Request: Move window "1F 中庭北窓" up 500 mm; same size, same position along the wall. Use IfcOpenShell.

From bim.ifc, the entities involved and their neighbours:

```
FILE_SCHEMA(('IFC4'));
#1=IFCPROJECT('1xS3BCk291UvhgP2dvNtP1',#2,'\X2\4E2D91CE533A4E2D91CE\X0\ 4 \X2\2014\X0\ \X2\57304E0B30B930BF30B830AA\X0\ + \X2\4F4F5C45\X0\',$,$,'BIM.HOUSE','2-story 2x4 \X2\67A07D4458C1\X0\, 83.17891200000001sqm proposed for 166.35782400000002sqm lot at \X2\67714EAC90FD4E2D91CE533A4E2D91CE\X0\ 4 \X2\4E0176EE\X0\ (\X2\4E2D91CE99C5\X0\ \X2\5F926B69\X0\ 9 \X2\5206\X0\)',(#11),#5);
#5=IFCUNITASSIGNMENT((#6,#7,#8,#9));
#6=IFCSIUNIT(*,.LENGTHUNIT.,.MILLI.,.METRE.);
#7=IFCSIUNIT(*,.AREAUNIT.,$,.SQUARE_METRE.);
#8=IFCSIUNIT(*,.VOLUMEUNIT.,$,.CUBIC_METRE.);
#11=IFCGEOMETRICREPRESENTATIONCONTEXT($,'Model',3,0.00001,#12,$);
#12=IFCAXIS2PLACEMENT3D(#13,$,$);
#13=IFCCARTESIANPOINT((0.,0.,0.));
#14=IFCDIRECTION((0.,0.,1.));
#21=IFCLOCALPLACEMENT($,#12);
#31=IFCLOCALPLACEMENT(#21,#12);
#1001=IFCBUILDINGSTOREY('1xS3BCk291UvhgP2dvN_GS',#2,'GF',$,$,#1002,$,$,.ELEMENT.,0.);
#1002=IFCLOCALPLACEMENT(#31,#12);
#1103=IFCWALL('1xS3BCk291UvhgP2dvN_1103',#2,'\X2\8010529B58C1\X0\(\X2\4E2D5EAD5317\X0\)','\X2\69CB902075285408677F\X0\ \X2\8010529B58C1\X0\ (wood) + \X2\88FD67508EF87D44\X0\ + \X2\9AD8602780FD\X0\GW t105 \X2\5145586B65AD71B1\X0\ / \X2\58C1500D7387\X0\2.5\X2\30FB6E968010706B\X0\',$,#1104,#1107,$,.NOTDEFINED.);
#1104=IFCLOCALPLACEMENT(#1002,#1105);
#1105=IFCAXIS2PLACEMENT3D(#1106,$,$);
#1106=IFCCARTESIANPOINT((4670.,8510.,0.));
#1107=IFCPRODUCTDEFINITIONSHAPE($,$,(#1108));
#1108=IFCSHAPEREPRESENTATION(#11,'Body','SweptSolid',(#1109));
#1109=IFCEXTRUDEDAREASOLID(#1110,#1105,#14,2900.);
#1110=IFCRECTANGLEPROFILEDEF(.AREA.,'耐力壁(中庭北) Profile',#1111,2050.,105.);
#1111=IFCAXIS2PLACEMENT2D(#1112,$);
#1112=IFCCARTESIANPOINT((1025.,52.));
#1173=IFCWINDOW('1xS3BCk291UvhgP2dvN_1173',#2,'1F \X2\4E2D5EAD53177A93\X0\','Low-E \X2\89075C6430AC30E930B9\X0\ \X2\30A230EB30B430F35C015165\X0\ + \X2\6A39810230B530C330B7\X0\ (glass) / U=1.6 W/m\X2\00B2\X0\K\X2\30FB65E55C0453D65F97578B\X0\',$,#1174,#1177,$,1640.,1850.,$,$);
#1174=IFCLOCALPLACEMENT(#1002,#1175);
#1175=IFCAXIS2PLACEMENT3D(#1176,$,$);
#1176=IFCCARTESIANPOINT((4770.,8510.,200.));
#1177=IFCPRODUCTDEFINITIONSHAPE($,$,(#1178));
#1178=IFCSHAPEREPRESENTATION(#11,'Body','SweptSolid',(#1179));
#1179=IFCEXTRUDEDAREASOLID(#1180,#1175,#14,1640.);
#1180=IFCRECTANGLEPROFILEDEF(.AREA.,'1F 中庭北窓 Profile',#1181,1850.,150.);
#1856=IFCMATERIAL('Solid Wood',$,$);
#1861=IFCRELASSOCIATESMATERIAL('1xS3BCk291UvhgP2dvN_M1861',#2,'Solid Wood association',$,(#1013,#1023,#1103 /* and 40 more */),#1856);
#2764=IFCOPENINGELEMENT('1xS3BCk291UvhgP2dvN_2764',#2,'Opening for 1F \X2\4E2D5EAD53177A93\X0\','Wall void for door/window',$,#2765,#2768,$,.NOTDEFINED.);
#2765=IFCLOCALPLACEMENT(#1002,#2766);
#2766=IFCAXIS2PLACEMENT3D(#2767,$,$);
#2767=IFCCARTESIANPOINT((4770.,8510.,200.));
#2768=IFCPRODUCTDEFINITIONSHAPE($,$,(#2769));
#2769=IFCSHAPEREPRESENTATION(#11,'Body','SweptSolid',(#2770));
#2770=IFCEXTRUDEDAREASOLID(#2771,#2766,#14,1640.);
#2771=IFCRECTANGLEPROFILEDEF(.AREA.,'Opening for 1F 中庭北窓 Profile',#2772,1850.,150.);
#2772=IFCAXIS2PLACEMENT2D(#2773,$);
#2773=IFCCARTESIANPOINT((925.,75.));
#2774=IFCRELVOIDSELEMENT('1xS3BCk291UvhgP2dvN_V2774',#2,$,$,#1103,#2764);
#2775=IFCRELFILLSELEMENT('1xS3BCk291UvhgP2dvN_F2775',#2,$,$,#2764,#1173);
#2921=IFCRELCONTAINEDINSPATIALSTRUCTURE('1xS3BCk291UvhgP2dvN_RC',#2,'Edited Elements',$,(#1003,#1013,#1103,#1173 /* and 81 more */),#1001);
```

```python
import numpy as np
import ifcopenshell
import ifcopenshell.api.geometry
import ifcopenshell.util.placement
import ifcopenshell.util.unit

model = ifcopenshell.open("bim.ifc")
unit_scale = ifcopenshell.util.unit.calculate_unit_scale(model)

window = model.by_id(1173)
opening = window.FillsVoids[0].RelatingOpeningElement
dz = 0.5 / unit_scale

shift = np.array([0.0, 0.0, dz])
# The window is not placed relative to its opening, so move both.
for product in (opening, window):
    matrix = ifcopenshell.util.placement.get_local_placement(product.ObjectPlacement)
    matrix[:3, 3] += shift
    ifcopenshell.api.geometry.edit_object_placement(model, product=product, matrix=matrix, is_si=False)

print(f"moved by {dz * unit_scale:+.3f} m")

model.write("bim_updated.ifc")
```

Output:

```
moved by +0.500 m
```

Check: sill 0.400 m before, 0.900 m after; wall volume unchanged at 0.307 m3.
